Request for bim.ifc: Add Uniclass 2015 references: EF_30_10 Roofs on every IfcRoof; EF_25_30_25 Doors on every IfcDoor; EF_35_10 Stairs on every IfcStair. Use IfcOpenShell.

First a look at what the model holds.

```python
import ifcopenshell

model = ifcopenshell.open("bim.ifc")
print(model.schema)
print("classifications:", [c.Name for c in model.by_type("IfcClassification")])
for ifc_class in ("IfcDoor", "IfcRoof", "IfcStair", "IfcWall", "IfcWindow"):
    print(ifc_class, len(model.by_type(ifc_class)))
```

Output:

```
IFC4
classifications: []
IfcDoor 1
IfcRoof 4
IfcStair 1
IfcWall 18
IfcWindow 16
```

```python
import ifcopenshell
import ifcopenshell.api.classification

model = ifcopenshell.open("bim.ifc")

system = ifcopenshell.api.classification.add_classification(model, classification="Uniclass 2015")

codes = {
    "IfcRoof": ("EF_30_10", "Roofs"),
    "IfcDoor": ("EF_25_30_25", "Doors"),
    "IfcStair": ("EF_35_10", "Stairs"),
}
for ifc_class, (code, name) in codes.items():
    products = model.by_type(ifc_class)
    ifcopenshell.api.classification.add_reference(
        model, products=products, classification=system, identification=code, name=name
    )
    print(code, len(products))

model.write("bim_edited.ifc")
```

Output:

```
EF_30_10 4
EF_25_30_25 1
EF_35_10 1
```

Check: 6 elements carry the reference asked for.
